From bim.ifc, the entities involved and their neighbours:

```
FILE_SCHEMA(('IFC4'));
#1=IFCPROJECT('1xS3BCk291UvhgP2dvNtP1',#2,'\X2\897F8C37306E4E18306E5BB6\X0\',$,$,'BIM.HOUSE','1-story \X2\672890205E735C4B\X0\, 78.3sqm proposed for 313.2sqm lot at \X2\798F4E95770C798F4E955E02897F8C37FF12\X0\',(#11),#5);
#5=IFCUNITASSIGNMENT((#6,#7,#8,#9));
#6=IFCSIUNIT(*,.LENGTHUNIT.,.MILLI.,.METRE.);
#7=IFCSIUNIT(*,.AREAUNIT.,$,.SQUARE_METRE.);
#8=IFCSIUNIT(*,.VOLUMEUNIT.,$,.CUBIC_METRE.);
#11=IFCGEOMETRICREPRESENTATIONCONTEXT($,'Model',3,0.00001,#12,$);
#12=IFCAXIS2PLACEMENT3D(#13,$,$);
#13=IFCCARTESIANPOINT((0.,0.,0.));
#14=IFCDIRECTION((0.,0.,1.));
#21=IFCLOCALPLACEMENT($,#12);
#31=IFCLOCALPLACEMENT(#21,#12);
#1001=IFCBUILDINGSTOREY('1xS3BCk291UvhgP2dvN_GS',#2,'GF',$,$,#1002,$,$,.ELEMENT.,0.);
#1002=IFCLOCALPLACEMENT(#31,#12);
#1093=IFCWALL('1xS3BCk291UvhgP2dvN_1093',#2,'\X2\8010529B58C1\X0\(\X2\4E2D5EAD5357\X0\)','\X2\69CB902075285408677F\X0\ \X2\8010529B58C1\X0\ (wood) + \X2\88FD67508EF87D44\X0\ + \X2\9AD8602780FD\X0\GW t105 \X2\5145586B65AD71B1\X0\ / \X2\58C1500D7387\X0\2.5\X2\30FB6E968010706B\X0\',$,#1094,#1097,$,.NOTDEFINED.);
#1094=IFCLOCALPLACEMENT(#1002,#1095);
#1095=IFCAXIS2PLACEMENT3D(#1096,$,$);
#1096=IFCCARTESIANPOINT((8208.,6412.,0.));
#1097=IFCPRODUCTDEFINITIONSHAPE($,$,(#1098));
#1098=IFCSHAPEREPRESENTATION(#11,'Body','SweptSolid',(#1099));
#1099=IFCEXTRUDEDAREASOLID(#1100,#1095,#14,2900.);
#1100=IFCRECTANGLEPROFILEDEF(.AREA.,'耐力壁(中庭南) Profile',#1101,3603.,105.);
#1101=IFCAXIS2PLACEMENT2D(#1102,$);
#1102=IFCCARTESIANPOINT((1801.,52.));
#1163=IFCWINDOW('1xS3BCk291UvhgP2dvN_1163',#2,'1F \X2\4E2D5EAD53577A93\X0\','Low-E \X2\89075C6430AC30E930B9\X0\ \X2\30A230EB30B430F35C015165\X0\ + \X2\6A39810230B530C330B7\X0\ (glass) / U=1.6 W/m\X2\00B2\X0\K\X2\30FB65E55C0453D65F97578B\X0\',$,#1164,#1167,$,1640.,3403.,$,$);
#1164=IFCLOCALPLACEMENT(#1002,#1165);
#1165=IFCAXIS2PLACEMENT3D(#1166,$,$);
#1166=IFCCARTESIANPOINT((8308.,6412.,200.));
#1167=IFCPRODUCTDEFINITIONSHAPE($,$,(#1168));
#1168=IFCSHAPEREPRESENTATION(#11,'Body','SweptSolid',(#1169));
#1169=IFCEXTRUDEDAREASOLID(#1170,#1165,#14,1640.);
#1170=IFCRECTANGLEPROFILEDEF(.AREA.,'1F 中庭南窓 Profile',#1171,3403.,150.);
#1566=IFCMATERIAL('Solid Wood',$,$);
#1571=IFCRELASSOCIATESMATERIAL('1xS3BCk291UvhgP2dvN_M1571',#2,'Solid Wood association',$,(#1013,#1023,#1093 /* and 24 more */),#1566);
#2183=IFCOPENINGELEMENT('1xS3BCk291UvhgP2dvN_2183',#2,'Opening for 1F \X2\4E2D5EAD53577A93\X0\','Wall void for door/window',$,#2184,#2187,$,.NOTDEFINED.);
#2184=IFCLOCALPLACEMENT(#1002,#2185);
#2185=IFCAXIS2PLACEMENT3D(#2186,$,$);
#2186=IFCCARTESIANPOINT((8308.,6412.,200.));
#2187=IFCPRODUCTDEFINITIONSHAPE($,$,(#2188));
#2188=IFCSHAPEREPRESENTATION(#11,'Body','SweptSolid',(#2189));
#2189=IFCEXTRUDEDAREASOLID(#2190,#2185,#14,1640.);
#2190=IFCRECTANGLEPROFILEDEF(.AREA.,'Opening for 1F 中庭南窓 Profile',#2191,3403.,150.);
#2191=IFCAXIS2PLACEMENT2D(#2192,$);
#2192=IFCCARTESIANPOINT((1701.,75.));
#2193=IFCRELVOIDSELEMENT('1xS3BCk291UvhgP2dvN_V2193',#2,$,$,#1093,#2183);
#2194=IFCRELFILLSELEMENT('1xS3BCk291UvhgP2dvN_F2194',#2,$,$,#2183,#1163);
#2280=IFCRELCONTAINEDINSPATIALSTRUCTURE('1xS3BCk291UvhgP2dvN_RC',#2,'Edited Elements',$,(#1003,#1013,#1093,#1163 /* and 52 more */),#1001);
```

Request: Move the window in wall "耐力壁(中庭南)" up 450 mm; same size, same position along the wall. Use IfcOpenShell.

```python
import numpy as np
import ifcopenshell
import ifcopenshell.api.geometry
import ifcopenshell.util.placement
import ifcopenshell.util.unit

model = ifcopenshell.open("bim.ifc")
unit_scale = ifcopenshell.util.unit.calculate_unit_scale(model)

window = model.by_guid("1xS3BCk291UvhgP2dvN_1163")
opening = window.FillsVoids[0].RelatingOpeningElement
dz = 0.45 / unit_scale

shift = np.array([0.0, 0.0, dz])
# The window is not placed relative to its opening, so move both.
for product in (opening, window):
    matrix = ifcopenshell.util.placement.get_local_placement(product.ObjectPlacement)
    matrix[:3, 3] += shift
    ifcopenshell.api.geometry.edit_object_placement(model, product=product, matrix=matrix, is_si=False)

print(f"moved by {dz * unit_scale:+.3f} m")

model.write("bim-out.ifc")
```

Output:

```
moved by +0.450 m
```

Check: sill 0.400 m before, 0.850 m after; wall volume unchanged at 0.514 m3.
